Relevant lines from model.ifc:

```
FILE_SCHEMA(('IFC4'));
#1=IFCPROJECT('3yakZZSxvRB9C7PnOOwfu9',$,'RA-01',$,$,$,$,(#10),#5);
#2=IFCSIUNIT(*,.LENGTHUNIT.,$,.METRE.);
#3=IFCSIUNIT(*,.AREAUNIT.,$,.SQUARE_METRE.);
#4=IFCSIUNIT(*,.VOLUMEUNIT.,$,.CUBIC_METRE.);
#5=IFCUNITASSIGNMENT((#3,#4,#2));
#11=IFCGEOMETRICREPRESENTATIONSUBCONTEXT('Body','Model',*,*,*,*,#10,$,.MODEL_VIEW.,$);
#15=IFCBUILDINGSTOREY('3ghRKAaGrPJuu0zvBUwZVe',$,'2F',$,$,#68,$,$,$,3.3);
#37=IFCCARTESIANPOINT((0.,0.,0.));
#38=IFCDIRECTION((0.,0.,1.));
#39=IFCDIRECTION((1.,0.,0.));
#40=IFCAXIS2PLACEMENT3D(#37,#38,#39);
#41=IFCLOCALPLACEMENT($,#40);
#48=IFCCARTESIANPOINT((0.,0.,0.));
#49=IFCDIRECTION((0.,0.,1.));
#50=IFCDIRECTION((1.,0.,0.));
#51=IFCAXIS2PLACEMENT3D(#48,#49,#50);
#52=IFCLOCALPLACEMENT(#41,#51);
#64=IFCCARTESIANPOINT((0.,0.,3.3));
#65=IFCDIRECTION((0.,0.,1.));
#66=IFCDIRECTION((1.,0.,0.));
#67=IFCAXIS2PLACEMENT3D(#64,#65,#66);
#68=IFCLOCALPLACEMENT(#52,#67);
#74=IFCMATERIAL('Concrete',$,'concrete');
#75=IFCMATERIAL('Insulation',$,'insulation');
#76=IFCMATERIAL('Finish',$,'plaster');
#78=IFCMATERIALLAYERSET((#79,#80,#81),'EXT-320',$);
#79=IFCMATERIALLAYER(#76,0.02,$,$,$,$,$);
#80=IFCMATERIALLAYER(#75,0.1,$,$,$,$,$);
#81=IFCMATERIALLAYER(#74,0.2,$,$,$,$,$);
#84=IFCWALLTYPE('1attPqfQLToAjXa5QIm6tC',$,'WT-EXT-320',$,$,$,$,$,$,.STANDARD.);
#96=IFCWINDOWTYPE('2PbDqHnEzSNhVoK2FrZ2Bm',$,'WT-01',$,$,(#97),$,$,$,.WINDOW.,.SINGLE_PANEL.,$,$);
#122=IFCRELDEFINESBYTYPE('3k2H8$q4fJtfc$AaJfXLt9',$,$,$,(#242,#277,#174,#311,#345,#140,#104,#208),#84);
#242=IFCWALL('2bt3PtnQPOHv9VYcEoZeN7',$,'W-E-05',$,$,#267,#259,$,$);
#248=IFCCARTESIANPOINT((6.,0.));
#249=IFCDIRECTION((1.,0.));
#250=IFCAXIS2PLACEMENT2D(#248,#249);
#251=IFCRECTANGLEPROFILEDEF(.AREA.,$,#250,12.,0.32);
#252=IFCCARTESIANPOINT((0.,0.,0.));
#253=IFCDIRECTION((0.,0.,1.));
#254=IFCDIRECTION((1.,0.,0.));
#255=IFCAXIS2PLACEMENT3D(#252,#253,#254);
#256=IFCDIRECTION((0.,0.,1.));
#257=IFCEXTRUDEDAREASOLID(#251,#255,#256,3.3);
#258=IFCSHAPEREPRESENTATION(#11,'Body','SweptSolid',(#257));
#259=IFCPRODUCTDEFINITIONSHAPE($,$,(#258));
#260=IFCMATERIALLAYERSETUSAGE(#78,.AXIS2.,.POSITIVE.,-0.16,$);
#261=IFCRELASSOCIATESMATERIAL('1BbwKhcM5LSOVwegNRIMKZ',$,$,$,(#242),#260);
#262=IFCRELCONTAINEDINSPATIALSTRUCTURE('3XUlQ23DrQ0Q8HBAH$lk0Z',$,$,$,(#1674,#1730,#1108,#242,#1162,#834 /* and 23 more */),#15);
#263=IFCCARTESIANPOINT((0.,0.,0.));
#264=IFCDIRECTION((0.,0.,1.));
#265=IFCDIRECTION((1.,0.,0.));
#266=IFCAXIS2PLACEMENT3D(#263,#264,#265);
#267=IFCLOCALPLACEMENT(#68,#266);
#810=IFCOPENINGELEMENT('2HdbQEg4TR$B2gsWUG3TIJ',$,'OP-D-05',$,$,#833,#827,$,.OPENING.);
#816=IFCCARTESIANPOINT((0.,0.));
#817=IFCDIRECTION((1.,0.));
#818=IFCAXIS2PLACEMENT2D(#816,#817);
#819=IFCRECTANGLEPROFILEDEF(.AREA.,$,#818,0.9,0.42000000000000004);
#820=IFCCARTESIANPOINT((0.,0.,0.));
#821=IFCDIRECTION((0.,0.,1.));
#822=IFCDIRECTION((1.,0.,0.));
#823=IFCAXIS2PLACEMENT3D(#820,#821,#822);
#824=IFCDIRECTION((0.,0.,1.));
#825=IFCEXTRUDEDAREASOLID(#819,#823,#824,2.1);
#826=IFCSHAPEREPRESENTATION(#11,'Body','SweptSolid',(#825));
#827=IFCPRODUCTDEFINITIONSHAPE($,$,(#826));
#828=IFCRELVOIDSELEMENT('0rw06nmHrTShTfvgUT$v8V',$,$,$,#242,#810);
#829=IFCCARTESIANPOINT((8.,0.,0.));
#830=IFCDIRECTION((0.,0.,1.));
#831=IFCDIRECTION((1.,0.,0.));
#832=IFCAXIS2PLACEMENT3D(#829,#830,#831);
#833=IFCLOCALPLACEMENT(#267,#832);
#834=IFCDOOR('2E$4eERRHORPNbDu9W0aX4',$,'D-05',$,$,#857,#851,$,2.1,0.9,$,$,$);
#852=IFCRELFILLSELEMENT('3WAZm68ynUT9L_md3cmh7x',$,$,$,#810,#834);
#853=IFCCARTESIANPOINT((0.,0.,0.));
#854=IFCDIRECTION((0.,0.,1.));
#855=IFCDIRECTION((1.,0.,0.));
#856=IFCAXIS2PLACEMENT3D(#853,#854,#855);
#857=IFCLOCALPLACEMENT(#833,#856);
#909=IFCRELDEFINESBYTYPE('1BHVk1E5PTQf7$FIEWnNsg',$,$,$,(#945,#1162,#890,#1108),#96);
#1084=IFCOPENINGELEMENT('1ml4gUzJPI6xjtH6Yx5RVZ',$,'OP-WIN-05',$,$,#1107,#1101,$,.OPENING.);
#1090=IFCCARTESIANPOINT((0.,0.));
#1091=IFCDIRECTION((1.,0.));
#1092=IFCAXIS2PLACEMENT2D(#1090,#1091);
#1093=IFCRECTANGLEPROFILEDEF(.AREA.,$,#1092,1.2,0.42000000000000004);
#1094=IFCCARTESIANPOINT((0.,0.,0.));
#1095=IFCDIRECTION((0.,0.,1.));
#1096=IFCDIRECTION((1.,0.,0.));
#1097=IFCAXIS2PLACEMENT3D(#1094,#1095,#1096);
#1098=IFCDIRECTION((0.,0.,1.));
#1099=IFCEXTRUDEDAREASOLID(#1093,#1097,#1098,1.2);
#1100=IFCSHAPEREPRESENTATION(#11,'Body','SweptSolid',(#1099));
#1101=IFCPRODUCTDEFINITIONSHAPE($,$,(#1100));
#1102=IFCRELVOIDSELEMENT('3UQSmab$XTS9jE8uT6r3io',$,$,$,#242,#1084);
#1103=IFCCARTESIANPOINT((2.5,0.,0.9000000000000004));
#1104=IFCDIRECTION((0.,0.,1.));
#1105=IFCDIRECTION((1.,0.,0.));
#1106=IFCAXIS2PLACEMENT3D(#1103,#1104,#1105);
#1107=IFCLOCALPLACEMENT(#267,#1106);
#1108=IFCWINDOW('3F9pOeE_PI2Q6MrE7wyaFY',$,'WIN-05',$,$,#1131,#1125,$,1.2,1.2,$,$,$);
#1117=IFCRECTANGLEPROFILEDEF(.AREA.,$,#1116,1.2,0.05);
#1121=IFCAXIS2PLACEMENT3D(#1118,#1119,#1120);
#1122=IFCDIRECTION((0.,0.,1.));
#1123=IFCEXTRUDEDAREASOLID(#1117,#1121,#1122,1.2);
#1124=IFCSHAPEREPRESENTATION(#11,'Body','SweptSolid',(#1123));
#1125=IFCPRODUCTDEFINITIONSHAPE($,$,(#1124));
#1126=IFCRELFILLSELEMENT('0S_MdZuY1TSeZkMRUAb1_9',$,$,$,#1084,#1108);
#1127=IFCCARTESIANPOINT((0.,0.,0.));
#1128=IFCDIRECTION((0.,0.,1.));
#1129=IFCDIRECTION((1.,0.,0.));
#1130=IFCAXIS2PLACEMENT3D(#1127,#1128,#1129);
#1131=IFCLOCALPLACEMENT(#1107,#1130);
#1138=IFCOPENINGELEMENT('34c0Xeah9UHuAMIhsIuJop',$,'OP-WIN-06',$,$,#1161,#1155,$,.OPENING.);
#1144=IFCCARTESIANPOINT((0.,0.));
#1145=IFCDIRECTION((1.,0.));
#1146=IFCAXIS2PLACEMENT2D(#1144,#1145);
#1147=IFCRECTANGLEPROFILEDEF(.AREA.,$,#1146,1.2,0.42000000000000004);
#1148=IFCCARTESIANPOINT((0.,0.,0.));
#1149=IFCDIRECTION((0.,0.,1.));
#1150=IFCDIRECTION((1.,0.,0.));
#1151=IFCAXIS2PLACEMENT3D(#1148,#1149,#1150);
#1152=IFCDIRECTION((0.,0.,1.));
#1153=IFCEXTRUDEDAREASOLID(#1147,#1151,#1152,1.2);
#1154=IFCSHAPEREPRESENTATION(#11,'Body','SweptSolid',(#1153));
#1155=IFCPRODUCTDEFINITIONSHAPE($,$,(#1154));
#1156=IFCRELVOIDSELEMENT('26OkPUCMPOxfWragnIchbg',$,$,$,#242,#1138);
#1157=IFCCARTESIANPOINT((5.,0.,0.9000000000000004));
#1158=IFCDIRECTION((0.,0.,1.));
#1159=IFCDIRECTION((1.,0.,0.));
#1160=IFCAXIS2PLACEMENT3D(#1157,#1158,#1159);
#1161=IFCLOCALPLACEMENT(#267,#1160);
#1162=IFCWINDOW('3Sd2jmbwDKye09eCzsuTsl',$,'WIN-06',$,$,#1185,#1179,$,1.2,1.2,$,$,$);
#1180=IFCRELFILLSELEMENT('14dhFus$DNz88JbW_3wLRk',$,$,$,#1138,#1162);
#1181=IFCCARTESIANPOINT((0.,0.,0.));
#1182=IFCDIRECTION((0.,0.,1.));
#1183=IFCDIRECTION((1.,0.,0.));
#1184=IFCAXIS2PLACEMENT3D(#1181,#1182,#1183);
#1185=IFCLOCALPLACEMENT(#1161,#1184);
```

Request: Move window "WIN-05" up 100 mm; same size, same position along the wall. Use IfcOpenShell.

```python
import numpy as np
import ifcopenshell
import ifcopenshell.api.geometry
import ifcopenshell.util.placement
import ifcopenshell.util.unit

model = ifcopenshell.open("model.ifc")
unit_scale = ifcopenshell.util.unit.calculate_unit_scale(model)

window = model.by_id(1108)
opening = window.FillsVoids[0].RelatingOpeningElement
dz = 0.1

shift = np.array([0.0, 0.0, dz])
# The window is placed relative to its opening, so it follows when the opening moves.
matrix = ifcopenshell.util.placement.get_local_placement(opening.ObjectPlacement)
matrix[:3, 3] += shift
ifcopenshell.api.geometry.edit_object_placement(
    model, product=opening, matrix=matrix, is_si=False, should_transform_children=True
)

print(f"moved by {dz * unit_scale:+.3f} m")

model.write("model_updated.ifc")
```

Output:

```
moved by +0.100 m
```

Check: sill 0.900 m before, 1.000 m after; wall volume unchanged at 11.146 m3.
